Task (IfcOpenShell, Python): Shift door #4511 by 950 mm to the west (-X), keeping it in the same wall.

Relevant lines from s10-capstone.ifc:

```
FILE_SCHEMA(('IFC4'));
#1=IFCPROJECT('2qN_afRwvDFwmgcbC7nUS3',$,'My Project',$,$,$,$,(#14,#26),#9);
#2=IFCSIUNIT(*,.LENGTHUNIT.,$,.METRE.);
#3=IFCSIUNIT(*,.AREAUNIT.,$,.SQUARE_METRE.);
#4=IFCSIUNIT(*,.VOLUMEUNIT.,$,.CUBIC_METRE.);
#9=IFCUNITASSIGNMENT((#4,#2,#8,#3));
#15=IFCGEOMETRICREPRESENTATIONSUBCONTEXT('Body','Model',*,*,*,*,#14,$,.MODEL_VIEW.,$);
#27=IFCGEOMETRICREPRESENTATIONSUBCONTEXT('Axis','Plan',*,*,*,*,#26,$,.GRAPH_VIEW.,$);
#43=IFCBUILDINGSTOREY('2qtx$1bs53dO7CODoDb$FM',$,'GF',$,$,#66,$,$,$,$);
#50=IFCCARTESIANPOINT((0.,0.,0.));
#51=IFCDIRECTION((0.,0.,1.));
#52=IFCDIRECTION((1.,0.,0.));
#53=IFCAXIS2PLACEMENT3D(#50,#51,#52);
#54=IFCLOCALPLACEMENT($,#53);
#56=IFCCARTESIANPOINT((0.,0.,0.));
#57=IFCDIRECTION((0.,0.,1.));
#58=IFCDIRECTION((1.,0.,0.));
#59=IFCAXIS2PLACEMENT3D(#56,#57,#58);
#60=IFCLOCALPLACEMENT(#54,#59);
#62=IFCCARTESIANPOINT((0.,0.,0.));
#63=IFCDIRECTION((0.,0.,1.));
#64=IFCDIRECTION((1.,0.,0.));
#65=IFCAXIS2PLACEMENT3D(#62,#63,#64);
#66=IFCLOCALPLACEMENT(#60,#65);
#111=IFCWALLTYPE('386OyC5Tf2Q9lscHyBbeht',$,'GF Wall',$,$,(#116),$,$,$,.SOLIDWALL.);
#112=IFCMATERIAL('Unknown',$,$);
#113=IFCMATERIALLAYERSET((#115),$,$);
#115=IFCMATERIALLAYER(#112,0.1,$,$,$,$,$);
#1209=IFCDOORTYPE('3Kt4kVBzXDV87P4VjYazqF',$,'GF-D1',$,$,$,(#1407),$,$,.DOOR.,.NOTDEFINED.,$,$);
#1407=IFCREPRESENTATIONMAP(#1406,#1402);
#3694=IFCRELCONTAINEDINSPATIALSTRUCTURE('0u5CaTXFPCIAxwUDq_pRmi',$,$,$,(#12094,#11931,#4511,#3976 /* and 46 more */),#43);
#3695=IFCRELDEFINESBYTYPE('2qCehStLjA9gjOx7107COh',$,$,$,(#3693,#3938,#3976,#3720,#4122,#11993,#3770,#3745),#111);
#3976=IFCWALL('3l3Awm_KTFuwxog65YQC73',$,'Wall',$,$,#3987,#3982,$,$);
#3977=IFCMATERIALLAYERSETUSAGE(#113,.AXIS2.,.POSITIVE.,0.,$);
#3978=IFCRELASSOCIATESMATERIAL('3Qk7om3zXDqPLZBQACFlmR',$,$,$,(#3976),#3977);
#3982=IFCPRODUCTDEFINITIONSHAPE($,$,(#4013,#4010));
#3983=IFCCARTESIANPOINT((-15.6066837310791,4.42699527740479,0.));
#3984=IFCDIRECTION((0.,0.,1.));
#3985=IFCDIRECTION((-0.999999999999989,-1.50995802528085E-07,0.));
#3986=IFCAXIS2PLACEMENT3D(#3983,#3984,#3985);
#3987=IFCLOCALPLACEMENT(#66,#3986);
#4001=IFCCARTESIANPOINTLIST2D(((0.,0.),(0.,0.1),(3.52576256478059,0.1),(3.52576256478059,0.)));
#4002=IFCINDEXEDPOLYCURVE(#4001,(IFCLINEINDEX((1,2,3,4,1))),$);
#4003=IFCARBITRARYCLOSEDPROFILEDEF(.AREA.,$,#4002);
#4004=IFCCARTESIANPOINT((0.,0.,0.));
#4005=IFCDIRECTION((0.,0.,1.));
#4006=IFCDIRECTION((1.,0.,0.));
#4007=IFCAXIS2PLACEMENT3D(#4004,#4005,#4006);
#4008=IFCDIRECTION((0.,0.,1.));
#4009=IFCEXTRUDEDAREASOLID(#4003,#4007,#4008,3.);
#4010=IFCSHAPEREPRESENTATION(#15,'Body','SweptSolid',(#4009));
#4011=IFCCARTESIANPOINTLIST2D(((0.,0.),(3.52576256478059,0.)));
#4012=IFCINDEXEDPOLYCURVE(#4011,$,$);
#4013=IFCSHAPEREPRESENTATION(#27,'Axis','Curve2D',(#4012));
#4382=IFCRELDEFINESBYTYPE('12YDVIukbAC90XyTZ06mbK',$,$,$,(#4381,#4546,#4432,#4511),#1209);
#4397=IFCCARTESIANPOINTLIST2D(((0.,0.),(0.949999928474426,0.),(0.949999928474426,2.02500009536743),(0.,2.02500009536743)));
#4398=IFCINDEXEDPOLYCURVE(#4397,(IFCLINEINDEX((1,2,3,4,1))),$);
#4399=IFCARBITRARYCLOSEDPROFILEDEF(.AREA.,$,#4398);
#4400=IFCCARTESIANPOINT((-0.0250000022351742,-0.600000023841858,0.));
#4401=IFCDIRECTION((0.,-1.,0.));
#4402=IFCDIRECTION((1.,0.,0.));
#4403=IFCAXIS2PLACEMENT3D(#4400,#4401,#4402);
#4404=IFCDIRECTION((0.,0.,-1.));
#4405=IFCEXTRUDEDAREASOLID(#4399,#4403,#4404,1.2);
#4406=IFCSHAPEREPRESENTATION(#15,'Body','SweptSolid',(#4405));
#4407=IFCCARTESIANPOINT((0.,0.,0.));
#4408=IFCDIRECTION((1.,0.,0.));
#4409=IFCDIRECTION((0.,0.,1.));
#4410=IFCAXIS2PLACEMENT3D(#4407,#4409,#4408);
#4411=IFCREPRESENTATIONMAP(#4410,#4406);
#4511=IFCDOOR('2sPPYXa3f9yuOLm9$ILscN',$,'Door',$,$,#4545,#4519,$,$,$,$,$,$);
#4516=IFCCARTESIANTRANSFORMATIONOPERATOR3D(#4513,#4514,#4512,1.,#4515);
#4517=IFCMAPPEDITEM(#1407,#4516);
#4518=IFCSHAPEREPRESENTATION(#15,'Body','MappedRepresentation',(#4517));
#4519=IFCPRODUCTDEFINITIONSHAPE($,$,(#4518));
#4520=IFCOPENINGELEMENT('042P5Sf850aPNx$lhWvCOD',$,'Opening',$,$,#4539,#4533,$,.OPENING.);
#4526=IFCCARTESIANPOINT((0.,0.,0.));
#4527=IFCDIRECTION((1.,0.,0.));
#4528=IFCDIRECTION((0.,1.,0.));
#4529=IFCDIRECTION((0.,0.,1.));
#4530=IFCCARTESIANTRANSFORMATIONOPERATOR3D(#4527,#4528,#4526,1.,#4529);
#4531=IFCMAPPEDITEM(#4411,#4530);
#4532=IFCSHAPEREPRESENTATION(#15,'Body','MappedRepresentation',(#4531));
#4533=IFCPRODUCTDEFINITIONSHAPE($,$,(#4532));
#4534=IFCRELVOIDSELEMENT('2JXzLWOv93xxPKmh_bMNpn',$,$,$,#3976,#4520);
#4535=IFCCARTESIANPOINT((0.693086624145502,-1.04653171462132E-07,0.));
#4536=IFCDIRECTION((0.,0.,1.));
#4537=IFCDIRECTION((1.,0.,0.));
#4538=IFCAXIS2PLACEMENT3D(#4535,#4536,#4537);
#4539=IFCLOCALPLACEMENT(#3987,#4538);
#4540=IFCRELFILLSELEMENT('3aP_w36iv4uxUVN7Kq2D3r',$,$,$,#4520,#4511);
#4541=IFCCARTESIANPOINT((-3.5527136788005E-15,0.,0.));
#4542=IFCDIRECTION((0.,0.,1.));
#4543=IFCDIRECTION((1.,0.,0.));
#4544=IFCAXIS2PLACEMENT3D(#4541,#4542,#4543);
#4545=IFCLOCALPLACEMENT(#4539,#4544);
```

```python
import ifcopenshell
import ifcopenshell.api.geometry
import ifcopenshell.util.placement
import ifcopenshell.util.unit

model = ifcopenshell.open("s10-capstone.ifc")
unit_scale = ifcopenshell.util.unit.calculate_unit_scale(model)

door = model.by_id(4511)
opening = door.FillsVoids[0].RelatingOpeningElement
wall = opening.VoidsElements[0].RelatingBuildingElement

wall_matrix = ifcopenshell.util.placement.get_local_placement(wall.ObjectPlacement)
shift = wall_matrix[:3, 0] * 0.95 / unit_scale
before = ifcopenshell.util.placement.get_local_placement(door.ObjectPlacement)[:3, 3].copy()

# The door is placed relative to its opening, so it follows when the opening moves.
matrix = ifcopenshell.util.placement.get_local_placement(opening.ObjectPlacement)
matrix[:3, 3] += shift
ifcopenshell.api.geometry.edit_object_placement(
    model, product=opening, matrix=matrix, is_si=False, should_transform_children=True
)

after = ifcopenshell.util.placement.get_local_placement(door.ObjectPlacement)[:3, 3]
print("door moved by", (after - before).round(3) + 0.0)

model.write("s10-capstone-out.ifc")
```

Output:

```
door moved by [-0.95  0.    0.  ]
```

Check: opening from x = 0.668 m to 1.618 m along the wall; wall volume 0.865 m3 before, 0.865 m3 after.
